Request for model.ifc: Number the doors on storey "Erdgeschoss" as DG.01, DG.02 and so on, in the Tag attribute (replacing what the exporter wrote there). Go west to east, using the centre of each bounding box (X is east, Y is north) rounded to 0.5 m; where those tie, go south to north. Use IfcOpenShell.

First a look at what the model holds.

```python
import ifcopenshell
import ifcopenshell.util.element
import ifcopenshell.util.placement

model = ifcopenshell.open("model.ifc")
print(model.schema)
storey = next(s for s in model.by_type("IfcBuildingStorey") if s.Name == "Erdgeschoss")
doors = [e for e in ifcopenshell.util.element.get_decomposition(storey) if e.is_a("IfcDoor")]
for e in sorted(doors, key=lambda e: e.id()):
    origin = ifcopenshell.util.placement.get_local_placement(e.ObjectPlacement)[:3, 3]
    print(e.id(), e.Tag, e.Name, origin.round(2) + 0.0, sep=" | ")
```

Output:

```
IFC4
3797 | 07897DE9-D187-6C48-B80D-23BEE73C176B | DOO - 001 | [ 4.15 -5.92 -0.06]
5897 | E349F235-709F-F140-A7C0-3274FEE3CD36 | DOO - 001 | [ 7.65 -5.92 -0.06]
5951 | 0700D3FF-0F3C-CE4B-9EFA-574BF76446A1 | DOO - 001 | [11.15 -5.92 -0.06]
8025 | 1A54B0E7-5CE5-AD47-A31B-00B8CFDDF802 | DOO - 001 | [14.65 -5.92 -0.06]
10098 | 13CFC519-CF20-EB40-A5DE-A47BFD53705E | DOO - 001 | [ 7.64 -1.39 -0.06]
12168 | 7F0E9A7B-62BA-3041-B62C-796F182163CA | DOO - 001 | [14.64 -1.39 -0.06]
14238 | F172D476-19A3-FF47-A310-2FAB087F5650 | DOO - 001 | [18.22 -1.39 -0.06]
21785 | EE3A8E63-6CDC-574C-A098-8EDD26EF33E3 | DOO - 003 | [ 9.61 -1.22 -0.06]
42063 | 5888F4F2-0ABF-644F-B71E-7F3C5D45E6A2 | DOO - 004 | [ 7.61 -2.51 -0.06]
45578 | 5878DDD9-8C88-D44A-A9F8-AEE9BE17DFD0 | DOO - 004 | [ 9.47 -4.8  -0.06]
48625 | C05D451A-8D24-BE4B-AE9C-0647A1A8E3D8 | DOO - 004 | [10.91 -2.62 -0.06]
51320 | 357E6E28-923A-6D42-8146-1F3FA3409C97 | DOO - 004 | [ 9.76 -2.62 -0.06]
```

```python
import ifcopenshell
import ifcopenshell.geom
import ifcopenshell.util.element
import ifcopenshell.util.shape

model = ifcopenshell.open("model.ifc")
settings = ifcopenshell.geom.settings()
settings.set("use-world-coords", True)


def centre(element):
    shape = ifcopenshell.geom.create_shape(settings, element)
    return ifcopenshell.util.shape.get_bbox_centroid(shape.geometry)


storey = next(s for s in model.by_type("IfcBuildingStorey") if s.Name == "Erdgeschoss")
doors = [e for e in ifcopenshell.util.element.get_decomposition(storey) if e.is_a("IfcDoor")]

# Insertion points can sit at a corner or the storey origin, so sort by the geometry (in metres).
centres = {e: centre(e) for e in doors}
doors.sort(key=lambda e: (round(centres[e][0] / 0.5), centres[e][1]))

for i, e in enumerate(doors, start=1):
    number = f"DG.{i:02d}"
    e.Tag = number
    print(e.id(), number)

model.write("model-out.ifc")
```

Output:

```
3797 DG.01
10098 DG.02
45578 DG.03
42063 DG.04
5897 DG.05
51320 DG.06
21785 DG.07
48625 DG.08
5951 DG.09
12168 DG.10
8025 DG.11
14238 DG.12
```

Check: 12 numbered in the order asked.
